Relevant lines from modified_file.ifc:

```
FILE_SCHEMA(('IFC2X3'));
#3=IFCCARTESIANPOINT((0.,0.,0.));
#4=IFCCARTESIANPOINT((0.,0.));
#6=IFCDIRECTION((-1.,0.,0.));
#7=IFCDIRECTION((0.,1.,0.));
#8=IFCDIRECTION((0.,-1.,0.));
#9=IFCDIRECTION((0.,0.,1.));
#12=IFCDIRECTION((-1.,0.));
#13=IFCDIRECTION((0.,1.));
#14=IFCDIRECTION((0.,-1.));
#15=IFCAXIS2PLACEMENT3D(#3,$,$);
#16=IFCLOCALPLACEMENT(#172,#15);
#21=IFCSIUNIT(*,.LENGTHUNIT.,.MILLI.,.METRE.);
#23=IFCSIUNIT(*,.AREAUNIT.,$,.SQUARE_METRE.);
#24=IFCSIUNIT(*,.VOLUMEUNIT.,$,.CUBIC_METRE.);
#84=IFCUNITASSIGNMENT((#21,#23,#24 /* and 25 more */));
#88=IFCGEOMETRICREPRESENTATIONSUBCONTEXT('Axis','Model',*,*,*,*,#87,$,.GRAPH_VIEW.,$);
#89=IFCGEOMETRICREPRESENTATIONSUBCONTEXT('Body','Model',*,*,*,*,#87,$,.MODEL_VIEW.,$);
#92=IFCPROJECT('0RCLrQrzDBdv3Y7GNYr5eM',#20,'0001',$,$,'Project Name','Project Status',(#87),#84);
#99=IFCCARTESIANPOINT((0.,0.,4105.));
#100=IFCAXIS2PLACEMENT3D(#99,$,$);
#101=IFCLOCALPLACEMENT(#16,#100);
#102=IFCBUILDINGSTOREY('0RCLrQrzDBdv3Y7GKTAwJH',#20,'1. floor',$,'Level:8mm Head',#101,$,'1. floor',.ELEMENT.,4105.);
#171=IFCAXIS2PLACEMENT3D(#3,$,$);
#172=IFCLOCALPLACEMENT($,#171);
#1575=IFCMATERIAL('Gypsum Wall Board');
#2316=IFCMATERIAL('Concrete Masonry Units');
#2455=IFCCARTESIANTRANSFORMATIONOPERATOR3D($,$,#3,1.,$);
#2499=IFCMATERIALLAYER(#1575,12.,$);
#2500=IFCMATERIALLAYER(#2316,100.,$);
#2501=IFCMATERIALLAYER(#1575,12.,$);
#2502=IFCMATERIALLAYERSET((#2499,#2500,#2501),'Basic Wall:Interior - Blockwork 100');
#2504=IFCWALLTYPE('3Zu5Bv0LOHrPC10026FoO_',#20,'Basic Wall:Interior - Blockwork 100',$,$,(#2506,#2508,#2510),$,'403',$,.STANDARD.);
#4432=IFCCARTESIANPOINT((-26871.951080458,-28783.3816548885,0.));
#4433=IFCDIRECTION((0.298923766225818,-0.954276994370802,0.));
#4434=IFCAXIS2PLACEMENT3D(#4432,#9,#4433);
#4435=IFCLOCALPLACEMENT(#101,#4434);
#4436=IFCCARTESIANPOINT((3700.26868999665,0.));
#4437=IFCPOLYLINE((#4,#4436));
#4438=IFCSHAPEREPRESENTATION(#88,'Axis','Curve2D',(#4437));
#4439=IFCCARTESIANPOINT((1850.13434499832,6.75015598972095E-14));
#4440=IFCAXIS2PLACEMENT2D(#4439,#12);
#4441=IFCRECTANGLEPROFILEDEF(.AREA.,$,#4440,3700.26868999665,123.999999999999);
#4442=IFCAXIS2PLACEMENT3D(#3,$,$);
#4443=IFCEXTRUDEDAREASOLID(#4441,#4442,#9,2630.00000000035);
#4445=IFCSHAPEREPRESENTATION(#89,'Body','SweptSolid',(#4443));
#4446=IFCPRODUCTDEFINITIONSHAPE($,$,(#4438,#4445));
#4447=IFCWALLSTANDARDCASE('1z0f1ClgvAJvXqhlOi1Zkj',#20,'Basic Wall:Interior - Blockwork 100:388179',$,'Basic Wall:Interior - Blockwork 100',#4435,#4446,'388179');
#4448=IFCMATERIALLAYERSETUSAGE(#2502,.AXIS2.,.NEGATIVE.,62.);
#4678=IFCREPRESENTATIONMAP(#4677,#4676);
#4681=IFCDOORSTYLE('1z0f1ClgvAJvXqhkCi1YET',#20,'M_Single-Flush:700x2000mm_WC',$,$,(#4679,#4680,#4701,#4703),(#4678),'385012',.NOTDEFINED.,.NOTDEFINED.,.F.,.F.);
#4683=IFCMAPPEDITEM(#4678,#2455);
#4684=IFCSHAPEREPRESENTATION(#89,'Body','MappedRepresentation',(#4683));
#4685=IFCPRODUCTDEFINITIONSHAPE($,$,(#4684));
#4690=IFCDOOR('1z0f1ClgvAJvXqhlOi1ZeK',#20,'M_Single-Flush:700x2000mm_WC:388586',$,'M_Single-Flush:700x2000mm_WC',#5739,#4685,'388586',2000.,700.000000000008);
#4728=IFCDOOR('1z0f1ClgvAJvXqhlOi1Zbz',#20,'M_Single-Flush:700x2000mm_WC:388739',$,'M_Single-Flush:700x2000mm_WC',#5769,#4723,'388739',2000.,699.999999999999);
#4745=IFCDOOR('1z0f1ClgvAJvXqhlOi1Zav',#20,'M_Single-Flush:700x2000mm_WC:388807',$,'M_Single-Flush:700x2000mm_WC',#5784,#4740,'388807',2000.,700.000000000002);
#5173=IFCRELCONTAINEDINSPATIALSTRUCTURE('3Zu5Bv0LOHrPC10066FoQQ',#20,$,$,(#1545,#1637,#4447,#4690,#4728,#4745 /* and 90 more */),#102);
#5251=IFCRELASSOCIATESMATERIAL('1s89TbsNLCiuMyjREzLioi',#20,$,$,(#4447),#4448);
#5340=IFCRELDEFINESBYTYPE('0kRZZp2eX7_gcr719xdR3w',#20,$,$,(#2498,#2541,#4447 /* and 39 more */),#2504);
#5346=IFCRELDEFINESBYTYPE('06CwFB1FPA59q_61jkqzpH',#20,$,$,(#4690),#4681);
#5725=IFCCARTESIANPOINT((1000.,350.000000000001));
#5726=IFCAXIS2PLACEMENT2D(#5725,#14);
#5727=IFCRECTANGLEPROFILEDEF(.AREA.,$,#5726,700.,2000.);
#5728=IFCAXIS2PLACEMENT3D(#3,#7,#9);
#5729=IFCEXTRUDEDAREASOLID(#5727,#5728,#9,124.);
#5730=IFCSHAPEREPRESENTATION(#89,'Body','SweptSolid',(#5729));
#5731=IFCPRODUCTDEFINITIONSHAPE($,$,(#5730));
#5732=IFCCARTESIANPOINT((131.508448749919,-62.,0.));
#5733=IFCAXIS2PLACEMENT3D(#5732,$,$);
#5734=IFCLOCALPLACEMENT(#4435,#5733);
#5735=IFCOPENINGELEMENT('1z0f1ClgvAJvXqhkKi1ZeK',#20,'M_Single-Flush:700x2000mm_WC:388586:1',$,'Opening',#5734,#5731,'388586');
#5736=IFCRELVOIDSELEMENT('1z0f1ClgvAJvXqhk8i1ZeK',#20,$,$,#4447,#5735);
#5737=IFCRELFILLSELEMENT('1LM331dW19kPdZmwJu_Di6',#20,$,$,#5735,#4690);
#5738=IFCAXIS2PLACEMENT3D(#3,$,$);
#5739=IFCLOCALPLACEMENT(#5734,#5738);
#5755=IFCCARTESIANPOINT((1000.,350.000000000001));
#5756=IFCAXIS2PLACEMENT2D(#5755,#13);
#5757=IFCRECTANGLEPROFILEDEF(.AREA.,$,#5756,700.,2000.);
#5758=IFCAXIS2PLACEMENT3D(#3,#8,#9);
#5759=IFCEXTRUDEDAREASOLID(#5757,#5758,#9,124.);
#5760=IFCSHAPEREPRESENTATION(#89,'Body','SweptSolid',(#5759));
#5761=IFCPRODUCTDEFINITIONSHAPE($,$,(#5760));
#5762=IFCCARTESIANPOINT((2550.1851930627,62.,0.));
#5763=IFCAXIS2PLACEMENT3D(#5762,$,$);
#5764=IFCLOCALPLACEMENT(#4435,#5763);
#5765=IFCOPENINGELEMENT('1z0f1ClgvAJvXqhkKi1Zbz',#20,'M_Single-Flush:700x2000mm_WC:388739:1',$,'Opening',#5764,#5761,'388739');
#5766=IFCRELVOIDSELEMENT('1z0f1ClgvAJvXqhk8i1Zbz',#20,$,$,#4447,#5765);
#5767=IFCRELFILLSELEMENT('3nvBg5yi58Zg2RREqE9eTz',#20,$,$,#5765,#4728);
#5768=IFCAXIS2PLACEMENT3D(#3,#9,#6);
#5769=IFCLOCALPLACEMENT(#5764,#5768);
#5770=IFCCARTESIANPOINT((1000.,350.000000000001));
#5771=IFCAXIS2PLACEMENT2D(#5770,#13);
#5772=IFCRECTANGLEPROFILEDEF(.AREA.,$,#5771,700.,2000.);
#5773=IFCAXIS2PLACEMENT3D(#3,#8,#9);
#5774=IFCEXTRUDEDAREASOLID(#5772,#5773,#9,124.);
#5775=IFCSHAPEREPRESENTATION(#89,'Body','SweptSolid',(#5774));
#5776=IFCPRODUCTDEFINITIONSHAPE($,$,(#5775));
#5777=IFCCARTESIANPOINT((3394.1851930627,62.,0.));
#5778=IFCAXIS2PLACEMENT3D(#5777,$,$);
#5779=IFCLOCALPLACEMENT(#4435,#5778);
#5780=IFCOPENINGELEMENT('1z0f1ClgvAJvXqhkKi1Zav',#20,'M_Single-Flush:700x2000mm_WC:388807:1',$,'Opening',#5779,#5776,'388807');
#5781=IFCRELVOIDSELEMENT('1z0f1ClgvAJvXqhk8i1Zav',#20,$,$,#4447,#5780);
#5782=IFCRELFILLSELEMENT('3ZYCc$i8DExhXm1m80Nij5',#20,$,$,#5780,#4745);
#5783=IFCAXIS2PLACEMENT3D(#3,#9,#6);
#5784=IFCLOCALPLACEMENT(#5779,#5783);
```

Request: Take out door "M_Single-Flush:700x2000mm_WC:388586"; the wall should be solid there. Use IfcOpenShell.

```python
import ifcopenshell
import ifcopenshell.api.feature
import ifcopenshell.api.root
import ifcopenshell.geom
import ifcopenshell.util.shape

model = ifcopenshell.open("modified_file.ifc")
settings = ifcopenshell.geom.settings()


def volume(element):
    """Net volume in cubic metres, openings subtracted."""
    shape = ifcopenshell.geom.create_shape(settings, element)
    return ifcopenshell.util.shape.get_volume(shape.geometry)


door = model.by_guid("1z0f1ClgvAJvXqhlOi1ZeK")
opening = door.FillsVoids[0].RelatingOpeningElement
wall = opening.VoidsElements[0].RelatingBuildingElement
before = volume(wall)

ifcopenshell.api.root.remove_product(model, product=door)
ifcopenshell.api.feature.remove_feature(model, feature=opening)

after = volume(wall)

print(f"wall volume {before:.3f} -> {after:.3f} m3")

model.write("modified_file_edited.ifc")
```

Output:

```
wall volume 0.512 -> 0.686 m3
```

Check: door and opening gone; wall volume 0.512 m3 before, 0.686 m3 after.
